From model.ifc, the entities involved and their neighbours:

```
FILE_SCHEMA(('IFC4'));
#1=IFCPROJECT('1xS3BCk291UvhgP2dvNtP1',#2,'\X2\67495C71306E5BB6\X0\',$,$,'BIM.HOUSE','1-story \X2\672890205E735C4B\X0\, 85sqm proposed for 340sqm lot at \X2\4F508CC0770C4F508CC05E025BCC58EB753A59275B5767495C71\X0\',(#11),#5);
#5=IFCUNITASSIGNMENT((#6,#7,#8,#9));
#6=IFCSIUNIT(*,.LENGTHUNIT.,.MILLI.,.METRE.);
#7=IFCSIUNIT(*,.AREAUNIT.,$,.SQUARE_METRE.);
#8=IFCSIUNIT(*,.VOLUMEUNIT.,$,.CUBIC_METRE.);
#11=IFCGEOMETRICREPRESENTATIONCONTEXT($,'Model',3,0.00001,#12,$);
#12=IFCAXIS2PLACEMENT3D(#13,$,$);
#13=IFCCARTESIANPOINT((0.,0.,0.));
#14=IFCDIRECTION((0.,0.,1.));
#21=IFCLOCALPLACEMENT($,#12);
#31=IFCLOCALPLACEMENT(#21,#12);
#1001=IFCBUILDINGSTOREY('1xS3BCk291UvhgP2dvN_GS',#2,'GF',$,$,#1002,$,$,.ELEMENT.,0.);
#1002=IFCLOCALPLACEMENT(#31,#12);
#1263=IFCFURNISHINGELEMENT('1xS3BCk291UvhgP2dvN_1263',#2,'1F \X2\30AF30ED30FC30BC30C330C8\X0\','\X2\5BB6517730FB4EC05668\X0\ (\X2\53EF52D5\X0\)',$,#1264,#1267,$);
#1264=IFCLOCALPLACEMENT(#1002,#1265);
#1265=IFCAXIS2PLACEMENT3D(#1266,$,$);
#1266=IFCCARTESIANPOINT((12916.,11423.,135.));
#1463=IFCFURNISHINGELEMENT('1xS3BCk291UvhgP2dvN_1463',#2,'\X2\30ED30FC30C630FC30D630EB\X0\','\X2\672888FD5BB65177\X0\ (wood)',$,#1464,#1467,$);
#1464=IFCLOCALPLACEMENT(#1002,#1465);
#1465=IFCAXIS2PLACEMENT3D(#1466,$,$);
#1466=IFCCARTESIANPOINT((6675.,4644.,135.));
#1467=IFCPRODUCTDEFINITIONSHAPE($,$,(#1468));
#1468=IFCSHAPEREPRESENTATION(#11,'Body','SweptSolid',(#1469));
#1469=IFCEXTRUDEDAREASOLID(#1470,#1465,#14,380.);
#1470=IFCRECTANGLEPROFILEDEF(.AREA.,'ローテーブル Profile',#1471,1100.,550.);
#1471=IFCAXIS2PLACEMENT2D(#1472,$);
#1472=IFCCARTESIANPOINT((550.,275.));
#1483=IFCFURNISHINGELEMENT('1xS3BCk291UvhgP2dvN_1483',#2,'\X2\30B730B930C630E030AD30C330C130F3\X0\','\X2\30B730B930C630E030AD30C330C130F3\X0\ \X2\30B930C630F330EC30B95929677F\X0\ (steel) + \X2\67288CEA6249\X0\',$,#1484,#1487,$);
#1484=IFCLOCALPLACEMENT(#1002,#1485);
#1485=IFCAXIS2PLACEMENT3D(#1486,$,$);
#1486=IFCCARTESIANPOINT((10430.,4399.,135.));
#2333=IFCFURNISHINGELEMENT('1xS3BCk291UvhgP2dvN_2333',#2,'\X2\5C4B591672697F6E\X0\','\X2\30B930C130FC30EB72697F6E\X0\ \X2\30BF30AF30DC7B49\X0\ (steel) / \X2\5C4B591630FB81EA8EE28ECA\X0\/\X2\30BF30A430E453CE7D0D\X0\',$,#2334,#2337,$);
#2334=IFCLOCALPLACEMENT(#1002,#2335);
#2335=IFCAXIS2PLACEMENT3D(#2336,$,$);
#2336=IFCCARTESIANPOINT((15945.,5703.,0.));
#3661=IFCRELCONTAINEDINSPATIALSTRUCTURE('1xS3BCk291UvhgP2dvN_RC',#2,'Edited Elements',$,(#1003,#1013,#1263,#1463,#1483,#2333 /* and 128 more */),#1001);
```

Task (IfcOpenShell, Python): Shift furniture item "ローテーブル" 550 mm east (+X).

```python
import ifcopenshell
import ifcopenshell.api.geometry
import ifcopenshell.util.placement
import ifcopenshell.util.unit

model = ifcopenshell.open("model.ifc")
unit_scale = ifcopenshell.util.unit.calculate_unit_scale(model)

item = model.by_id(1463)
matrix = ifcopenshell.util.placement.get_local_placement(item.ObjectPlacement)
matrix[0, 3] += 0.55 / unit_scale
ifcopenshell.api.geometry.edit_object_placement(model, product=item, matrix=matrix, is_si=False)

print(ifcopenshell.util.placement.get_local_placement(item.ObjectPlacement).round(3) + 0.0)

model.write("model_v2.ifc")
```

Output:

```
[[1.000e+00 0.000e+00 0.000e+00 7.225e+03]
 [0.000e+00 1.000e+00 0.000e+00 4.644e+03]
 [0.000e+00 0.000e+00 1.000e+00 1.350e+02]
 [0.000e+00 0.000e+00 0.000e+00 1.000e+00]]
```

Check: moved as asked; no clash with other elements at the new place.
